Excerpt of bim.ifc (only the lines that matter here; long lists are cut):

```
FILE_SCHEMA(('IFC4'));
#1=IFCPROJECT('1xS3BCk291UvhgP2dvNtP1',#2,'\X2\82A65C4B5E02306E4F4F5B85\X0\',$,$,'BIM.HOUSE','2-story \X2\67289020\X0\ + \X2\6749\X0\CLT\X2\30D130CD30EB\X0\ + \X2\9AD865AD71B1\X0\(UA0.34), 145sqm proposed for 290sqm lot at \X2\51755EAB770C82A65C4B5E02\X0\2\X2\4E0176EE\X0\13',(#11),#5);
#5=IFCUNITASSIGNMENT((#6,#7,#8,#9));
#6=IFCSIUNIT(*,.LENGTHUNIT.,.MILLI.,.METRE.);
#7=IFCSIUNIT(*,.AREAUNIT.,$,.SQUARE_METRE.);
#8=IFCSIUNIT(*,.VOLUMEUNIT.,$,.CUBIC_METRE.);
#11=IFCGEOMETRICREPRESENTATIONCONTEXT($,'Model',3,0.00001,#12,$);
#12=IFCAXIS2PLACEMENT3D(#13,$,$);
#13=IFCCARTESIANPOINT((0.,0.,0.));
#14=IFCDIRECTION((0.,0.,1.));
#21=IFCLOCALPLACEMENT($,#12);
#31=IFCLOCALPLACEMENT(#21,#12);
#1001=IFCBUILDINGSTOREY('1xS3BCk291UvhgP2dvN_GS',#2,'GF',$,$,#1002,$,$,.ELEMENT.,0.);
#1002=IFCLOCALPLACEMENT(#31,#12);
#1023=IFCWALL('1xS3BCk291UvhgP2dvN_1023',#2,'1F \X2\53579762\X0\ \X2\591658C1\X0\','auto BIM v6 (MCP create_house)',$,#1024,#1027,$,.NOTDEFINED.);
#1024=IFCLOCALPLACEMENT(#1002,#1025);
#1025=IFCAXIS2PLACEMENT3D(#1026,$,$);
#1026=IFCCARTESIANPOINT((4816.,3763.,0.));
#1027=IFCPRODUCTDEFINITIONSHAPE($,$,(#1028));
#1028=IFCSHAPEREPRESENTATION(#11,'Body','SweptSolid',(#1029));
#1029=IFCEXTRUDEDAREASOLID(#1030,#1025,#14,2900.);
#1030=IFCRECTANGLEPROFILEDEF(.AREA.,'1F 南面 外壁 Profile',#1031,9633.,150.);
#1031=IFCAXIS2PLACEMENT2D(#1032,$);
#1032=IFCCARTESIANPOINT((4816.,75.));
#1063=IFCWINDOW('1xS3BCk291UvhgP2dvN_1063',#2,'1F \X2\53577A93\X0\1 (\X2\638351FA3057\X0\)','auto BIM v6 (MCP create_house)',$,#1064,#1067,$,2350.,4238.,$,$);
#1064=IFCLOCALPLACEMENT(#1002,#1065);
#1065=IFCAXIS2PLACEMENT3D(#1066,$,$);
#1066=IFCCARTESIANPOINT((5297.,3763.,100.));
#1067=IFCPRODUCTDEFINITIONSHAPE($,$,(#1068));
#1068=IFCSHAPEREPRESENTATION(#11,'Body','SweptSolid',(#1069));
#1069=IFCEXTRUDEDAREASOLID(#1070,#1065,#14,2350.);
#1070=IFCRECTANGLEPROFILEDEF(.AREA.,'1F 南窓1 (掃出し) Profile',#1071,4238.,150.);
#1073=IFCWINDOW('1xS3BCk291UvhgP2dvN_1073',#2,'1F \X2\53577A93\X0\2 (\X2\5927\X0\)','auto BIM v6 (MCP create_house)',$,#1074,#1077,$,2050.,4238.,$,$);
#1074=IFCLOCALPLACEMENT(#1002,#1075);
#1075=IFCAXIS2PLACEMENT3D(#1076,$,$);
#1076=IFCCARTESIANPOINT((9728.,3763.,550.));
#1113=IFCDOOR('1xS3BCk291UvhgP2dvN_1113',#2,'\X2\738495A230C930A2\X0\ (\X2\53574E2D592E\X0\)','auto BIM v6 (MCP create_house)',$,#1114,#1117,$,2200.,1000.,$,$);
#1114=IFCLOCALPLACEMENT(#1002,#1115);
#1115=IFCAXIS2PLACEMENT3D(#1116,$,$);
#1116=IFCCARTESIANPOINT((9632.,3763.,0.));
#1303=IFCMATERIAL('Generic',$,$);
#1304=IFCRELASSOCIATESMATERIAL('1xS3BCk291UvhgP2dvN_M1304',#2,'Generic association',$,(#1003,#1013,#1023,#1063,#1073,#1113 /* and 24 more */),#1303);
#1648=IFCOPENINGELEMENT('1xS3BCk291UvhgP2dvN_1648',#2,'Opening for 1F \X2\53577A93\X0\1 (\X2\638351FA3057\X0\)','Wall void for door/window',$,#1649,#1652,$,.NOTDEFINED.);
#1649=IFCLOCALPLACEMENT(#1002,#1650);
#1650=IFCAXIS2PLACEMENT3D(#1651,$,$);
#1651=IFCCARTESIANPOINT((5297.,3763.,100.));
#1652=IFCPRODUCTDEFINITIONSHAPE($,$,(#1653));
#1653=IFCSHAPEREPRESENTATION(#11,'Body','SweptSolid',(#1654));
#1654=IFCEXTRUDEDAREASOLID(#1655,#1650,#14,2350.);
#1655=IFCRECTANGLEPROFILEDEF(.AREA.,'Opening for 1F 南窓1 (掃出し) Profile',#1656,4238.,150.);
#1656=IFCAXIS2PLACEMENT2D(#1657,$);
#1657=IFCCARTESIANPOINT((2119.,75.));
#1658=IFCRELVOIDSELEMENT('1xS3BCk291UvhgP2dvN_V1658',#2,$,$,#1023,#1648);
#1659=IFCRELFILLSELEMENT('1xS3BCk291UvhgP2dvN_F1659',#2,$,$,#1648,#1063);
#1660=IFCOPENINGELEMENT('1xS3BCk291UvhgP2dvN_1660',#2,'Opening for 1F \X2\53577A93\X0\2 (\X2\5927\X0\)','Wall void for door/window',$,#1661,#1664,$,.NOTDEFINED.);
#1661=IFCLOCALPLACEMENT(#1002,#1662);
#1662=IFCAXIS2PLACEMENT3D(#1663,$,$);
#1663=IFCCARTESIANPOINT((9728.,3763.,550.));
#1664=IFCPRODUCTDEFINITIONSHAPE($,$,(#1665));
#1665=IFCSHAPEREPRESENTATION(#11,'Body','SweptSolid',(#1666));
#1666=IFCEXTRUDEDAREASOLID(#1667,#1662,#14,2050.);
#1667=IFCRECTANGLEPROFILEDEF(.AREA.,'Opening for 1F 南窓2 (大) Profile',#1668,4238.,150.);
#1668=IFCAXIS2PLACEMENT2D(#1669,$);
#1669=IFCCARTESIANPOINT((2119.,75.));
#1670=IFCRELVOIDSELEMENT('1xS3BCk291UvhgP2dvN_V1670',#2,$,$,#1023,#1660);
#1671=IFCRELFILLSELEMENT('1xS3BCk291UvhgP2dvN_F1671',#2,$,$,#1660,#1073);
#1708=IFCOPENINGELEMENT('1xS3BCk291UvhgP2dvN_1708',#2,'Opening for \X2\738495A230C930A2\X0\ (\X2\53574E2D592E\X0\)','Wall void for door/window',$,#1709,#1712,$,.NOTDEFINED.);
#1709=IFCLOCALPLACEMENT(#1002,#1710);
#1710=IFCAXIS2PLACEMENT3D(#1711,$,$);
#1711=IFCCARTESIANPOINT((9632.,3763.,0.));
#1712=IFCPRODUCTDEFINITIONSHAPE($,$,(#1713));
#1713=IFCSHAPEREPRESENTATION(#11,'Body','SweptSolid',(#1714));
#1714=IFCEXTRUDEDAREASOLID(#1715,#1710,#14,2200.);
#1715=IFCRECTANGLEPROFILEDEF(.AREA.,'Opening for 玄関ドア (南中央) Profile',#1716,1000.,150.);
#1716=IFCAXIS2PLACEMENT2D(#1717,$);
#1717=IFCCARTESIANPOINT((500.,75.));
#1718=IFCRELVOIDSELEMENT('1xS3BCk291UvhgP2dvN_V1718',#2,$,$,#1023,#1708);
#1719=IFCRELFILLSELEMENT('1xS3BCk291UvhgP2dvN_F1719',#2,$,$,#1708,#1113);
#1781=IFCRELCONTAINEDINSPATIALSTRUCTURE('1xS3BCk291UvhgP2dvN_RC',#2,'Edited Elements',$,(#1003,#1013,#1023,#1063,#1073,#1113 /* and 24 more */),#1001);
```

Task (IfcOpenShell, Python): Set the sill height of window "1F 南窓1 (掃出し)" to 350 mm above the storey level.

```python
import numpy as np
import ifcopenshell
import ifcopenshell.api.geometry
import ifcopenshell.geom
import ifcopenshell.util.element
import ifcopenshell.util.placement
import ifcopenshell.util.shape
import ifcopenshell.util.unit

model = ifcopenshell.open("bim.ifc")
unit_scale = ifcopenshell.util.unit.calculate_unit_scale(model)

window = model.by_guid("1xS3BCk291UvhgP2dvN_1063")
opening = window.FillsVoids[0].RelatingOpeningElement
storey = ifcopenshell.util.element.get_container(window, ifc_class="IfcBuildingStorey")
level = ifcopenshell.util.placement.get_local_placement(storey.ObjectPlacement)[2, 3]

# The opening's origin need not be at the sill, so measure its lowest point.
shape = ifcopenshell.geom.create_shape(ifcopenshell.geom.settings(), opening)
bottom = ifcopenshell.util.shape.get_shape_bottom_elevation(shape, shape.geometry) / unit_scale
dz = level + 350.0 - bottom

shift = np.array([0.0, 0.0, dz])
# The window is not placed relative to its opening, so move both.
for product in (opening, window):
    matrix = ifcopenshell.util.placement.get_local_placement(product.ObjectPlacement)
    matrix[:3, 3] += shift
    ifcopenshell.api.geometry.edit_object_placement(model, product=product, matrix=matrix, is_si=False)

print(f"moved by {dz * unit_scale:+.3f} m")

model.write("bim_updated.ifc")
```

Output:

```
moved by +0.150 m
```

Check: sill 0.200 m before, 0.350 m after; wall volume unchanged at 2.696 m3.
